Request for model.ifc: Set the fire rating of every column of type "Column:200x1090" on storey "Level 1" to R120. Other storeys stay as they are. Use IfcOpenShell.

First a look at what the model holds.

```python
import ifcopenshell
import ifcopenshell.util.element

model = ifcopenshell.open("model.ifc")
print(model.schema)
storey = next(s for s in model.by_type("IfcBuildingStorey") if s.Name == "Level 1")
columns = [e for e in ifcopenshell.util.element.get_decomposition(storey) if e.is_a("IfcColumn")]
seen = {}
for e in columns:
    element_type = ifcopenshell.util.element.get_type(e)
    key = (element_type.Name if element_type != e and element_type else None, ifcopenshell.util.element.get_pset(e, "Pset_ColumnCommon", "FireRating"))
    seen[key] = seen.get(key, 0) + 1
for (name, value), count in sorted(seen.items(), key=str):
    print(count, "x", name, "|", value)
```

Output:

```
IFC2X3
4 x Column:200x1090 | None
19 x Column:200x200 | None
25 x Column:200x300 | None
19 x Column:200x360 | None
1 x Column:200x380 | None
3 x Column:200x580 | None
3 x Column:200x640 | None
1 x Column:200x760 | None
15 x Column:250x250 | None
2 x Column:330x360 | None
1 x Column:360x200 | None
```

```python
import ifcopenshell
import ifcopenshell.api.pset
import ifcopenshell.util.element

model = ifcopenshell.open("model.ifc")

storey = next(s for s in model.by_type("IfcBuildingStorey") if s.Name == "Level 1")
columns = [e for e in ifcopenshell.util.element.get_decomposition(storey) if e.is_a("IfcColumn")]

count = 0
for e in columns:
    element_type = ifcopenshell.util.element.get_type(e)
    if element_type in (None, e) or element_type.Name != "Column:200x1090":
        continue
    # add_pset returns the element's existing set when there is one.
    pset = ifcopenshell.api.pset.add_pset(model, product=e, name="Pset_ColumnCommon")
    ifcopenshell.api.pset.edit_pset(model, pset=pset, properties={"FireRating": "R120"})
    count += 1

print(count, "columns updated")

model.write("model_rev.ifc")
```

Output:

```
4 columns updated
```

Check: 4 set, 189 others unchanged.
